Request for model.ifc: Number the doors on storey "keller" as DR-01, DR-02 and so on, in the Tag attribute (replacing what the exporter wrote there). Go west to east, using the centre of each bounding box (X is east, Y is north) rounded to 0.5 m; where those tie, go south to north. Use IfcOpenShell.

First a look at what the model holds.

```python
import ifcopenshell
import ifcopenshell.util.element
import ifcopenshell.util.placement

model = ifcopenshell.open("model.ifc")
print(model.schema)
storey = next(s for s in model.by_type("IfcBuildingStorey") if s.Name == "keller")
doors = [e for e in ifcopenshell.util.element.get_decomposition(storey) if e.is_a("IfcDoor")]
for e in sorted(doors, key=lambda e: e.id()):
    origin = ifcopenshell.util.placement.get_local_placement(e.ObjectPlacement)[:3, 3]
    print(e.id(), e.Tag, e.Name, origin.round(2) + 0.0, sep=" | ")
```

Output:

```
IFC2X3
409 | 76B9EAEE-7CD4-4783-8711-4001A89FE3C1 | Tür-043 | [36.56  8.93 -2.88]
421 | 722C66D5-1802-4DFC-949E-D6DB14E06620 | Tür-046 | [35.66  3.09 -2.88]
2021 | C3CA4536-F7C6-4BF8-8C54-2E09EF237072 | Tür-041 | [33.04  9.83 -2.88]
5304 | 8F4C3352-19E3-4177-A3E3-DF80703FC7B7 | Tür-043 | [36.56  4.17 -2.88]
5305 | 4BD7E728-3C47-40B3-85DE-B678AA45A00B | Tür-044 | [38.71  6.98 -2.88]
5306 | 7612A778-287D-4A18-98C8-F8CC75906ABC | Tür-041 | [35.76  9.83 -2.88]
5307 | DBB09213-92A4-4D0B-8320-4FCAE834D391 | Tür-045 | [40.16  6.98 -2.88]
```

```python
import ifcopenshell
import ifcopenshell.geom
import ifcopenshell.util.element
import ifcopenshell.util.shape

model = ifcopenshell.open("model.ifc")
settings = ifcopenshell.geom.settings()
settings.set("use-world-coords", True)


def centre(element):
    shape = ifcopenshell.geom.create_shape(settings, element)
    return ifcopenshell.util.shape.get_bbox_centroid(shape.geometry)


storey = next(s for s in model.by_type("IfcBuildingStorey") if s.Name == "keller")
doors = [e for e in ifcopenshell.util.element.get_decomposition(storey) if e.is_a("IfcDoor")]

# Insertion points can sit at a corner or the storey origin, so sort by the geometry (in metres).
centres = {e: centre(e) for e in doors}
doors.sort(key=lambda e: (round(centres[e][0] / 0.5), centres[e][1]))

for i, e in enumerate(doors, start=1):
    number = f"DR-{i:02d}"
    e.Tag = number
    print(e.id(), number)

model.write("model_rev.ifc")
```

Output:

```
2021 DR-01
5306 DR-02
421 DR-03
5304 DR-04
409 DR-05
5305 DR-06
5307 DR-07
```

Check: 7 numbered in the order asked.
